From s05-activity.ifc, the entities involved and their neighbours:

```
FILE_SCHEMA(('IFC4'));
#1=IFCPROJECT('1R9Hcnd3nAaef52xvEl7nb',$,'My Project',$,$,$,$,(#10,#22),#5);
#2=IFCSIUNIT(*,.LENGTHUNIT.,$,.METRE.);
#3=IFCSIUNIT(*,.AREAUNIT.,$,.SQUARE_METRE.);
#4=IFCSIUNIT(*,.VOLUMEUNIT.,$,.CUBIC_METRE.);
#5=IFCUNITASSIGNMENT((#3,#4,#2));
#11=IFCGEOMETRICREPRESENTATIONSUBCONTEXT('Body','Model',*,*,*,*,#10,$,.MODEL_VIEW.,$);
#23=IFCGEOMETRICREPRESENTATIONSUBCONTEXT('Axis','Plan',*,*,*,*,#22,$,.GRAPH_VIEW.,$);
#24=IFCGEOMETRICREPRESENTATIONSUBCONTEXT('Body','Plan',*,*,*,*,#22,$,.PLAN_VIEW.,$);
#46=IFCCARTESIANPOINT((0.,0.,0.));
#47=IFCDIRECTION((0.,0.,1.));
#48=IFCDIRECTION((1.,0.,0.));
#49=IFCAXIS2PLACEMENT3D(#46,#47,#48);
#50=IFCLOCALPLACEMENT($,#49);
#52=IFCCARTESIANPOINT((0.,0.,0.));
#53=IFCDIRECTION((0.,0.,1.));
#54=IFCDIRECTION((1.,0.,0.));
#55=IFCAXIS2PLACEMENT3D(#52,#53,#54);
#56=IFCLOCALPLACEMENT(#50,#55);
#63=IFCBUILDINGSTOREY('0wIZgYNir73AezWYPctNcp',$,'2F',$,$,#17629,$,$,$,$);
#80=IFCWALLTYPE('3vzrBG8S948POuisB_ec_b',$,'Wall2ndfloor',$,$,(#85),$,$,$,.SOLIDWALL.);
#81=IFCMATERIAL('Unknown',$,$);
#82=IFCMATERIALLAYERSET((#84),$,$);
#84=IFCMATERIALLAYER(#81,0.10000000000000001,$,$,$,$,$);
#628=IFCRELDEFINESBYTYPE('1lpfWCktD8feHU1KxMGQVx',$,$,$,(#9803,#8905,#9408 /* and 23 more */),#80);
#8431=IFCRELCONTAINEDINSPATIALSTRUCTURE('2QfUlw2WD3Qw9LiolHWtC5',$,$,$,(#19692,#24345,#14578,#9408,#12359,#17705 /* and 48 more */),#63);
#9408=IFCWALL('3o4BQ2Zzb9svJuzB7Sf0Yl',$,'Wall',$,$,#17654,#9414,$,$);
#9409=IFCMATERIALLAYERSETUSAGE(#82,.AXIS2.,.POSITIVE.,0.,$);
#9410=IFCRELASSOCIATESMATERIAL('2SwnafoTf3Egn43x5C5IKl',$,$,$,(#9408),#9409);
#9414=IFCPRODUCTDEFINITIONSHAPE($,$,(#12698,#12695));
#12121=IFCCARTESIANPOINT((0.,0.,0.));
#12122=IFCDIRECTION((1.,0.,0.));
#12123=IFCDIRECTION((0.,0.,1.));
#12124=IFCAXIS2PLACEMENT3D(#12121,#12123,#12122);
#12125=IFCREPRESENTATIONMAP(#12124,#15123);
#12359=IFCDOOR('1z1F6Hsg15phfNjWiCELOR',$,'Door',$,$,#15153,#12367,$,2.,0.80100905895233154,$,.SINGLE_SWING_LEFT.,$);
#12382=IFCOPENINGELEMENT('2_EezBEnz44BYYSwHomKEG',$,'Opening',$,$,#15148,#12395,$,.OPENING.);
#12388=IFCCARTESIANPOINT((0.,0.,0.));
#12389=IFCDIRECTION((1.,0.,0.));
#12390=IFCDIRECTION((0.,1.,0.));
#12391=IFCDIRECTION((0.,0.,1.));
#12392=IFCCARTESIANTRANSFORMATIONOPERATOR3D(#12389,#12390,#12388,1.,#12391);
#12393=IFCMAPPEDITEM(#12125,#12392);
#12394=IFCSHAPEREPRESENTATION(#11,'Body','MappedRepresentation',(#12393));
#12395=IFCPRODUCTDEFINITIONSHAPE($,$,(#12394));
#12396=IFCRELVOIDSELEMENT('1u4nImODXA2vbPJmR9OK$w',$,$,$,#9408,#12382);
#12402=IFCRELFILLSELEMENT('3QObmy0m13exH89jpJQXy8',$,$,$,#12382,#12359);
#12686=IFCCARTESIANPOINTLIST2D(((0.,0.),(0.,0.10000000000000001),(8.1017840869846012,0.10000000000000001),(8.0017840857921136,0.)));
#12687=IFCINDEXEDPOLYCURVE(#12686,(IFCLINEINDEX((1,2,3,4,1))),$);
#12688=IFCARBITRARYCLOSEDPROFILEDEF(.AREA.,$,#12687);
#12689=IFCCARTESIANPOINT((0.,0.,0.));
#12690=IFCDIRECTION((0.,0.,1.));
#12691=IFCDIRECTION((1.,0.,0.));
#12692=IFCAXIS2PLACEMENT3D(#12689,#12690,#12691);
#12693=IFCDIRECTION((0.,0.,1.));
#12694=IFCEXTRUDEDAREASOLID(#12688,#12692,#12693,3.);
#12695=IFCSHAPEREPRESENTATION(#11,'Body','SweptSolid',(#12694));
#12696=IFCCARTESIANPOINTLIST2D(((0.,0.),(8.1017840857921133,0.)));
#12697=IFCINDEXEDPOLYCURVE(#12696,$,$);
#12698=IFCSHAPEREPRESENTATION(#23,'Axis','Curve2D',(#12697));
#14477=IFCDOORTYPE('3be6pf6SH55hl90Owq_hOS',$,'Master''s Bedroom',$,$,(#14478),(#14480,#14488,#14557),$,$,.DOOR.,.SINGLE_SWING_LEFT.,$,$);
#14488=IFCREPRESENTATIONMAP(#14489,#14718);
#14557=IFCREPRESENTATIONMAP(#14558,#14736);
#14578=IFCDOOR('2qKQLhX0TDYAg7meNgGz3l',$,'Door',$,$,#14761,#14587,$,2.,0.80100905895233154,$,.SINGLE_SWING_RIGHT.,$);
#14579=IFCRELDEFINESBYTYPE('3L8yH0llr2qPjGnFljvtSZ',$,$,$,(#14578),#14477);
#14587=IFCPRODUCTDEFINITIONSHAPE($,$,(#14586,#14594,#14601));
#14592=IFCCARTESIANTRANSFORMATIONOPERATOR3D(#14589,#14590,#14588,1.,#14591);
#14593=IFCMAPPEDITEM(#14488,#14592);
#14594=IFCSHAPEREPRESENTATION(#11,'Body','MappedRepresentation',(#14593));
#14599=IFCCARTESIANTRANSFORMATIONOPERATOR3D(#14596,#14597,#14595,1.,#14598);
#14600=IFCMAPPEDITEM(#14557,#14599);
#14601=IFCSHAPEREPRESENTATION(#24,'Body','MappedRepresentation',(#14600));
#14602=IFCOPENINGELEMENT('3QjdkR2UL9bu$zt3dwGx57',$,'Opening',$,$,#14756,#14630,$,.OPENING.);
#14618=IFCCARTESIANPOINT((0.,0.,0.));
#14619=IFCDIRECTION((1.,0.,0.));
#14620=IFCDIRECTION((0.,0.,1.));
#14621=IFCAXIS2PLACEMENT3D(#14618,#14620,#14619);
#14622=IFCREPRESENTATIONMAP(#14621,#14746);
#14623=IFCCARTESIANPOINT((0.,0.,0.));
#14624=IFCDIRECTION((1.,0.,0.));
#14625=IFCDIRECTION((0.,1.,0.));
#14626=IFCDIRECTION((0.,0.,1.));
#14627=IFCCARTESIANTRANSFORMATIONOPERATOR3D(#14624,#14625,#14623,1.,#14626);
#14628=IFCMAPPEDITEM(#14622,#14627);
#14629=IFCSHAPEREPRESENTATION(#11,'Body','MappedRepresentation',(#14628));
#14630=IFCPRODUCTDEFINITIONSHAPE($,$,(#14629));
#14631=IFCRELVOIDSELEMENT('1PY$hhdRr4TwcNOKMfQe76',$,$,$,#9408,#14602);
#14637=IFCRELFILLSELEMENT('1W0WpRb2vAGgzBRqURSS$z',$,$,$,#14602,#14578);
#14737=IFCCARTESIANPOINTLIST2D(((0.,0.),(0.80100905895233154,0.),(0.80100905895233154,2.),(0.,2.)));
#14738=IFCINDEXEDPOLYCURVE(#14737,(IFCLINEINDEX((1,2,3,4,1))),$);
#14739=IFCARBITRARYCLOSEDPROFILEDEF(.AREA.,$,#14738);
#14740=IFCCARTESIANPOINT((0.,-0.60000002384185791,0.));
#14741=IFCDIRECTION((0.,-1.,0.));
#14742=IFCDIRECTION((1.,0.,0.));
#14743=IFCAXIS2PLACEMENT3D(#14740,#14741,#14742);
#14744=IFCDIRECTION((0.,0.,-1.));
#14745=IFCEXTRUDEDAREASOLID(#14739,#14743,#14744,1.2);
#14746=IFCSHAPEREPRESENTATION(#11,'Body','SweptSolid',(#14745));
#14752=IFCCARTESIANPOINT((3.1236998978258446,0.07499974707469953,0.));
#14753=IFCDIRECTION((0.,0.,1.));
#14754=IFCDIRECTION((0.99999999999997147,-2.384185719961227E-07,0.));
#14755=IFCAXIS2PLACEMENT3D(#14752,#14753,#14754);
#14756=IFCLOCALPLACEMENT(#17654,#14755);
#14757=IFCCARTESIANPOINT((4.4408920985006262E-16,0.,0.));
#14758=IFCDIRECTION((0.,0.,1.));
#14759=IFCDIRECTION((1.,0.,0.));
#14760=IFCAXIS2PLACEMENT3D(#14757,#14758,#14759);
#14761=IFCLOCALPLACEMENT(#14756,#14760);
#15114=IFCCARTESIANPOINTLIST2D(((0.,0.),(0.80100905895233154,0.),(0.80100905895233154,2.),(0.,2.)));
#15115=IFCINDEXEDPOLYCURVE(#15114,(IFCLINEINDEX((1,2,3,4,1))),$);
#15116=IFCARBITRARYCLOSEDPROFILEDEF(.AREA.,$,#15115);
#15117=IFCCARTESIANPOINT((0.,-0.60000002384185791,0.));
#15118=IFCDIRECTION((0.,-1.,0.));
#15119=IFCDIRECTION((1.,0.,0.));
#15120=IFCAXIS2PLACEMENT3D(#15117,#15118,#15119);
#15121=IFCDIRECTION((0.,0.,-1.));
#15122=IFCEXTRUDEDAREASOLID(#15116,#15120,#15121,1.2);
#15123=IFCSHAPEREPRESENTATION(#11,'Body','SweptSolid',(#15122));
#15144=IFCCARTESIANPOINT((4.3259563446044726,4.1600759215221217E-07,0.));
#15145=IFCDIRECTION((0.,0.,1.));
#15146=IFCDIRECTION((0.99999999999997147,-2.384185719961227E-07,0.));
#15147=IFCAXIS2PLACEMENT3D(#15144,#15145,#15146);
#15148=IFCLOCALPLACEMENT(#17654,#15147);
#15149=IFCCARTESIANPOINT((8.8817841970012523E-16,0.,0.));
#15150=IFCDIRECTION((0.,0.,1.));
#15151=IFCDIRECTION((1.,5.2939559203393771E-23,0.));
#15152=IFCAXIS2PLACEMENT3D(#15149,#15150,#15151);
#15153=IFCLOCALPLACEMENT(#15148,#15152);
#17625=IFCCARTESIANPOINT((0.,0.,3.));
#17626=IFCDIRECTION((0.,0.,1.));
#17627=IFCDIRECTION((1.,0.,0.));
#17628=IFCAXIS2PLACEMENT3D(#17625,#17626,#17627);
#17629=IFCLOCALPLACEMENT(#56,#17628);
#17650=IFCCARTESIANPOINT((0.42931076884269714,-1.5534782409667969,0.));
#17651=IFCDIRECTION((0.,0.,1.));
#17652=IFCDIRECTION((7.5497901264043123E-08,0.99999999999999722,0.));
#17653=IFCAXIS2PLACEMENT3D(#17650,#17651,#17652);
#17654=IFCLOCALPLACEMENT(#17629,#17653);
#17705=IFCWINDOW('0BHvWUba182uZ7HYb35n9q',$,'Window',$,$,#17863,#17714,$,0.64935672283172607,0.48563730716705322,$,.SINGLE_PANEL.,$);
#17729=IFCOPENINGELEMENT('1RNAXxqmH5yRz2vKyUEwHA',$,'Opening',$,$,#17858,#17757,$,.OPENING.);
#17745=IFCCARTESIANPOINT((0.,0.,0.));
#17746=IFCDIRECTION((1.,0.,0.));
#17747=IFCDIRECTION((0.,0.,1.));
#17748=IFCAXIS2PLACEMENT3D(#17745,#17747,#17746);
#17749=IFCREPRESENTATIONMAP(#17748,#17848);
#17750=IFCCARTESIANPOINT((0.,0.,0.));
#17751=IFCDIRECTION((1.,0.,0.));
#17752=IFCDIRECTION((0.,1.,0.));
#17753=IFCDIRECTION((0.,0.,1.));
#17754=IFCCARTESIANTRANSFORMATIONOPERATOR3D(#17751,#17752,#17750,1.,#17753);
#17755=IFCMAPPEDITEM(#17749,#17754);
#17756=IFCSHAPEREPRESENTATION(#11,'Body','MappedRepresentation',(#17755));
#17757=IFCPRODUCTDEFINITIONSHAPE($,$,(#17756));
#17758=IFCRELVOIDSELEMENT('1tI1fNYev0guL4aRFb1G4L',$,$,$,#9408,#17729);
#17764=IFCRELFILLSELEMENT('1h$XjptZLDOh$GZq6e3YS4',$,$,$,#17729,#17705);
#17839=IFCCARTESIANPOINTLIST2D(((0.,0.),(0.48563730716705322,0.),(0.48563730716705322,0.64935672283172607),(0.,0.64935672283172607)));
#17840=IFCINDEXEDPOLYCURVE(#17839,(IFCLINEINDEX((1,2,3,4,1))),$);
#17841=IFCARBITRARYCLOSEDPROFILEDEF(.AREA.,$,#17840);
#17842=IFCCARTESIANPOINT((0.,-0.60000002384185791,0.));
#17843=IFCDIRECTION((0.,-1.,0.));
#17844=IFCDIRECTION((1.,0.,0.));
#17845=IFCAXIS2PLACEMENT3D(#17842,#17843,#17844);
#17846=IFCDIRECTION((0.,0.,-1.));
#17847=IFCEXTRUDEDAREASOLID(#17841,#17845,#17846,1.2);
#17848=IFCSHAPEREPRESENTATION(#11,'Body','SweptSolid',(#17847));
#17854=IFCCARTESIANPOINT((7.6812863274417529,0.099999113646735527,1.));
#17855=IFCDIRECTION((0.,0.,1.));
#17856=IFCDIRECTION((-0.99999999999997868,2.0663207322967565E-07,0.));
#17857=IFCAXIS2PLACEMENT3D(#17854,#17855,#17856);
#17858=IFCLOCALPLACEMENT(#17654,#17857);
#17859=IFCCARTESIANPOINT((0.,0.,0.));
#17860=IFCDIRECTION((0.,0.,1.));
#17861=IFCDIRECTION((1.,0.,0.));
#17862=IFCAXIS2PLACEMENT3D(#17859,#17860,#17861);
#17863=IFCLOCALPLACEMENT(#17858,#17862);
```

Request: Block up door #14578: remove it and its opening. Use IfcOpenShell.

```python
import ifcopenshell
import ifcopenshell.api.feature
import ifcopenshell.api.root
import ifcopenshell.geom
import ifcopenshell.util.shape

model = ifcopenshell.open("s05-activity.ifc")
settings = ifcopenshell.geom.settings()


def volume(element):
    """Net volume in cubic metres, openings subtracted."""
    shape = ifcopenshell.geom.create_shape(settings, element)
    return ifcopenshell.util.shape.get_volume(shape.geometry)


door = model.by_guid("2qKQLhX0TDYAg7meNgGz3l")
opening = door.FillsVoids[0].RelatingOpeningElement
wall = opening.VoidsElements[0].RelatingBuildingElement
before = volume(wall)

ifcopenshell.api.root.remove_product(model, product=door)
ifcopenshell.api.feature.remove_feature(model, feature=opening)

after = volume(wall)

print(f"wall volume {before:.3f} -> {after:.3f} m3")

model.write("s05-activity_edited.ifc")
```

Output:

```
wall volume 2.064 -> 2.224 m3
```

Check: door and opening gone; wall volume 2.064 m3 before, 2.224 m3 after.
